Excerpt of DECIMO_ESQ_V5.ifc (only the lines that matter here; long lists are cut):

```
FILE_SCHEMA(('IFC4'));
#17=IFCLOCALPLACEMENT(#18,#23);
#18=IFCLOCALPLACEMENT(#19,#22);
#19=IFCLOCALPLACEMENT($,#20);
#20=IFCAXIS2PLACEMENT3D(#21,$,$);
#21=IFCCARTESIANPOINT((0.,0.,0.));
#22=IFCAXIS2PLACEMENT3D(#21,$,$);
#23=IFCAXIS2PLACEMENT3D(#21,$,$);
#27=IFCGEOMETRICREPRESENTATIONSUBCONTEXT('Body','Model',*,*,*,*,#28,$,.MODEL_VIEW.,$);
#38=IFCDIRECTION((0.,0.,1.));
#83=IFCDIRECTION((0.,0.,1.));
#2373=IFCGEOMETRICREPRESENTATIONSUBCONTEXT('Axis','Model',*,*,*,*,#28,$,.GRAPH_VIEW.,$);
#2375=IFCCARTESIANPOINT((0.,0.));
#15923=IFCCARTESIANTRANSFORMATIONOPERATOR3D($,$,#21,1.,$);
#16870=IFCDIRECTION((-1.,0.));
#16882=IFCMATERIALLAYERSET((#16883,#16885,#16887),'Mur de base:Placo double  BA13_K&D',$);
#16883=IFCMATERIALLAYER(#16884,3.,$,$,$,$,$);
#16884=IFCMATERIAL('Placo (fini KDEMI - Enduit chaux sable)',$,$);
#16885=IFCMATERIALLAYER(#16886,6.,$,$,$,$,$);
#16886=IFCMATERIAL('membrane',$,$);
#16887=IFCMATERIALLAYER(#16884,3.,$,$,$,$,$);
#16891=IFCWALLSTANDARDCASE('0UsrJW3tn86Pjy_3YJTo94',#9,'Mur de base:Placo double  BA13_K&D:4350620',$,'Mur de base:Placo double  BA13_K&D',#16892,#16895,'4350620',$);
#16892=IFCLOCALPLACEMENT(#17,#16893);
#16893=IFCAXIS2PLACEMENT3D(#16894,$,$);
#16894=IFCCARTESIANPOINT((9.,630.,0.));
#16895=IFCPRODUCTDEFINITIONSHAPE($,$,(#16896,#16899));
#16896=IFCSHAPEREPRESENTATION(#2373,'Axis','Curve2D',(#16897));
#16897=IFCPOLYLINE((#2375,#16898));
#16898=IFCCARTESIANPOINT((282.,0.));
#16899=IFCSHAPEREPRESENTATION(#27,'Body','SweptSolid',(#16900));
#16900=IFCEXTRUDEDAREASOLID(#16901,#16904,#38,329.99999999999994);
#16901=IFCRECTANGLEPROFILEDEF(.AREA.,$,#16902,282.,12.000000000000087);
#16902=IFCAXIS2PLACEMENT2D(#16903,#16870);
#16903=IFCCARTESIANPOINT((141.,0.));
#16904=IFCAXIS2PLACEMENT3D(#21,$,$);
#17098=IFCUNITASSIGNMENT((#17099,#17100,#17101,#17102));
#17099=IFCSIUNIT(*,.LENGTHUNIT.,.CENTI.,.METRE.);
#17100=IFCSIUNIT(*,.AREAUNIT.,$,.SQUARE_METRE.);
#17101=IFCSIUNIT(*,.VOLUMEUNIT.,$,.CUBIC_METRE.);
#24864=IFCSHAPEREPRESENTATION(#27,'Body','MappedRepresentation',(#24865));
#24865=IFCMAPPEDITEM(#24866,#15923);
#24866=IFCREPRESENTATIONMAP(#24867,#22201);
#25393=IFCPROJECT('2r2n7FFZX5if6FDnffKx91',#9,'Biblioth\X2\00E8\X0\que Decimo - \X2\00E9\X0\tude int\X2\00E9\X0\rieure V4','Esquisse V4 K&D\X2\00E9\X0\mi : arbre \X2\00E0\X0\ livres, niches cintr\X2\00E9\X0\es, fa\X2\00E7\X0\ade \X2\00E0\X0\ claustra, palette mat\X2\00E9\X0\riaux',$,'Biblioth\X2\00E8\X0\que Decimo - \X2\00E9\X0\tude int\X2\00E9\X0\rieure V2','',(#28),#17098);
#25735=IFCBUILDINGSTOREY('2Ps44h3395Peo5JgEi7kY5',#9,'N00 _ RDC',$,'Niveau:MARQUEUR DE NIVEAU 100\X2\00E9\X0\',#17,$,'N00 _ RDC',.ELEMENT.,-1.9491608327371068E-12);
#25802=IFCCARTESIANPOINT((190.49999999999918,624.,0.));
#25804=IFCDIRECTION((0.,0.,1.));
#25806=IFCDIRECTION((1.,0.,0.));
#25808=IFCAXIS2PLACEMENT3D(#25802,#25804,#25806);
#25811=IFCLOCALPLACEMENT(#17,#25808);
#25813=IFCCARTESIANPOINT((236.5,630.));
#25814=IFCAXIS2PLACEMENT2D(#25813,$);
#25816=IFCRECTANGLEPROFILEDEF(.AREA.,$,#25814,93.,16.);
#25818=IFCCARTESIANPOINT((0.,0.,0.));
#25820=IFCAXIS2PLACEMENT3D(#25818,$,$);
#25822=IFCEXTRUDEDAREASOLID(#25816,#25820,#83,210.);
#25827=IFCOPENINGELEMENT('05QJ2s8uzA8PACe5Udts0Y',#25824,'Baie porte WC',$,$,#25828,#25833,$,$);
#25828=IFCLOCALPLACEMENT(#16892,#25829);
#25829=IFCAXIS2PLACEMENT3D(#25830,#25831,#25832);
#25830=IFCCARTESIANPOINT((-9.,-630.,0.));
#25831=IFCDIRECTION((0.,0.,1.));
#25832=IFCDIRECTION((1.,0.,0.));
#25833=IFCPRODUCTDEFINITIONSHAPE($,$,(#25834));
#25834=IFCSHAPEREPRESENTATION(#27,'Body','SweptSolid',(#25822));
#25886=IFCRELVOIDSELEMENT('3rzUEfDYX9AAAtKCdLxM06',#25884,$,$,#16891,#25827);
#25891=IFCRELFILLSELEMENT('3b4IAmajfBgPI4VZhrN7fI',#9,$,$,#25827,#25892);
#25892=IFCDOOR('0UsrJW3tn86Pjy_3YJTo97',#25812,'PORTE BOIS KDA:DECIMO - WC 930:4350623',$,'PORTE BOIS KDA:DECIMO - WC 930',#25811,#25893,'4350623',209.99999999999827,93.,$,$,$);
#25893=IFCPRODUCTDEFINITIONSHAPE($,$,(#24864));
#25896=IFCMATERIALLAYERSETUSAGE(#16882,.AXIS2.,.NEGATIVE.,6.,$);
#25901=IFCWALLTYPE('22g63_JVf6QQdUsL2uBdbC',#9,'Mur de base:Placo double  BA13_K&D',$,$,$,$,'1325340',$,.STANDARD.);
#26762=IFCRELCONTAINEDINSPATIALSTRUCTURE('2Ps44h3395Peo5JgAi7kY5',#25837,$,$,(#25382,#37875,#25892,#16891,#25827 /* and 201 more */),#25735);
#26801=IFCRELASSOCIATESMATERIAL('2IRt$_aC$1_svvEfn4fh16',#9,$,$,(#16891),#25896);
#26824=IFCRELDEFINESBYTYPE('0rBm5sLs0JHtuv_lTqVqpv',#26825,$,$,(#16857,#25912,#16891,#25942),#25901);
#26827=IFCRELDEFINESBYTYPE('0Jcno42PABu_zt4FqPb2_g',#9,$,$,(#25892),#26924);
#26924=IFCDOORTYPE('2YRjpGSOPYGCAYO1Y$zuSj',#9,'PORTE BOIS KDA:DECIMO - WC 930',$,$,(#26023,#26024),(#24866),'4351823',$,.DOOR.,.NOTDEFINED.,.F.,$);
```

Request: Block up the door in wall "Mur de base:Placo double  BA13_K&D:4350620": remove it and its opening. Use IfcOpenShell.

```python
import ifcopenshell
import ifcopenshell.api.feature
import ifcopenshell.api.root
import ifcopenshell.geom
import ifcopenshell.util.shape

model = ifcopenshell.open("DECIMO_ESQ_V5.ifc")
settings = ifcopenshell.geom.settings()


def volume(element):
    """Net volume in cubic metres, openings subtracted."""
    shape = ifcopenshell.geom.create_shape(settings, element)
    return ifcopenshell.util.shape.get_volume(shape.geometry)


door = model.by_guid("0UsrJW3tn86Pjy_3YJTo97")
opening = door.FillsVoids[0].RelatingOpeningElement
wall = opening.VoidsElements[0].RelatingBuildingElement
before = volume(wall)

ifcopenshell.api.root.remove_product(model, product=door)
ifcopenshell.api.feature.remove_feature(model, feature=opening)

after = volume(wall)

print(f"wall volume {before:.3f} -> {after:.3f} m3")

model.write("DECIMO_ESQ_V5_rev.ifc")
```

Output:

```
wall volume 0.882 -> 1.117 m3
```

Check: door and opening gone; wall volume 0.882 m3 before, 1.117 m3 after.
